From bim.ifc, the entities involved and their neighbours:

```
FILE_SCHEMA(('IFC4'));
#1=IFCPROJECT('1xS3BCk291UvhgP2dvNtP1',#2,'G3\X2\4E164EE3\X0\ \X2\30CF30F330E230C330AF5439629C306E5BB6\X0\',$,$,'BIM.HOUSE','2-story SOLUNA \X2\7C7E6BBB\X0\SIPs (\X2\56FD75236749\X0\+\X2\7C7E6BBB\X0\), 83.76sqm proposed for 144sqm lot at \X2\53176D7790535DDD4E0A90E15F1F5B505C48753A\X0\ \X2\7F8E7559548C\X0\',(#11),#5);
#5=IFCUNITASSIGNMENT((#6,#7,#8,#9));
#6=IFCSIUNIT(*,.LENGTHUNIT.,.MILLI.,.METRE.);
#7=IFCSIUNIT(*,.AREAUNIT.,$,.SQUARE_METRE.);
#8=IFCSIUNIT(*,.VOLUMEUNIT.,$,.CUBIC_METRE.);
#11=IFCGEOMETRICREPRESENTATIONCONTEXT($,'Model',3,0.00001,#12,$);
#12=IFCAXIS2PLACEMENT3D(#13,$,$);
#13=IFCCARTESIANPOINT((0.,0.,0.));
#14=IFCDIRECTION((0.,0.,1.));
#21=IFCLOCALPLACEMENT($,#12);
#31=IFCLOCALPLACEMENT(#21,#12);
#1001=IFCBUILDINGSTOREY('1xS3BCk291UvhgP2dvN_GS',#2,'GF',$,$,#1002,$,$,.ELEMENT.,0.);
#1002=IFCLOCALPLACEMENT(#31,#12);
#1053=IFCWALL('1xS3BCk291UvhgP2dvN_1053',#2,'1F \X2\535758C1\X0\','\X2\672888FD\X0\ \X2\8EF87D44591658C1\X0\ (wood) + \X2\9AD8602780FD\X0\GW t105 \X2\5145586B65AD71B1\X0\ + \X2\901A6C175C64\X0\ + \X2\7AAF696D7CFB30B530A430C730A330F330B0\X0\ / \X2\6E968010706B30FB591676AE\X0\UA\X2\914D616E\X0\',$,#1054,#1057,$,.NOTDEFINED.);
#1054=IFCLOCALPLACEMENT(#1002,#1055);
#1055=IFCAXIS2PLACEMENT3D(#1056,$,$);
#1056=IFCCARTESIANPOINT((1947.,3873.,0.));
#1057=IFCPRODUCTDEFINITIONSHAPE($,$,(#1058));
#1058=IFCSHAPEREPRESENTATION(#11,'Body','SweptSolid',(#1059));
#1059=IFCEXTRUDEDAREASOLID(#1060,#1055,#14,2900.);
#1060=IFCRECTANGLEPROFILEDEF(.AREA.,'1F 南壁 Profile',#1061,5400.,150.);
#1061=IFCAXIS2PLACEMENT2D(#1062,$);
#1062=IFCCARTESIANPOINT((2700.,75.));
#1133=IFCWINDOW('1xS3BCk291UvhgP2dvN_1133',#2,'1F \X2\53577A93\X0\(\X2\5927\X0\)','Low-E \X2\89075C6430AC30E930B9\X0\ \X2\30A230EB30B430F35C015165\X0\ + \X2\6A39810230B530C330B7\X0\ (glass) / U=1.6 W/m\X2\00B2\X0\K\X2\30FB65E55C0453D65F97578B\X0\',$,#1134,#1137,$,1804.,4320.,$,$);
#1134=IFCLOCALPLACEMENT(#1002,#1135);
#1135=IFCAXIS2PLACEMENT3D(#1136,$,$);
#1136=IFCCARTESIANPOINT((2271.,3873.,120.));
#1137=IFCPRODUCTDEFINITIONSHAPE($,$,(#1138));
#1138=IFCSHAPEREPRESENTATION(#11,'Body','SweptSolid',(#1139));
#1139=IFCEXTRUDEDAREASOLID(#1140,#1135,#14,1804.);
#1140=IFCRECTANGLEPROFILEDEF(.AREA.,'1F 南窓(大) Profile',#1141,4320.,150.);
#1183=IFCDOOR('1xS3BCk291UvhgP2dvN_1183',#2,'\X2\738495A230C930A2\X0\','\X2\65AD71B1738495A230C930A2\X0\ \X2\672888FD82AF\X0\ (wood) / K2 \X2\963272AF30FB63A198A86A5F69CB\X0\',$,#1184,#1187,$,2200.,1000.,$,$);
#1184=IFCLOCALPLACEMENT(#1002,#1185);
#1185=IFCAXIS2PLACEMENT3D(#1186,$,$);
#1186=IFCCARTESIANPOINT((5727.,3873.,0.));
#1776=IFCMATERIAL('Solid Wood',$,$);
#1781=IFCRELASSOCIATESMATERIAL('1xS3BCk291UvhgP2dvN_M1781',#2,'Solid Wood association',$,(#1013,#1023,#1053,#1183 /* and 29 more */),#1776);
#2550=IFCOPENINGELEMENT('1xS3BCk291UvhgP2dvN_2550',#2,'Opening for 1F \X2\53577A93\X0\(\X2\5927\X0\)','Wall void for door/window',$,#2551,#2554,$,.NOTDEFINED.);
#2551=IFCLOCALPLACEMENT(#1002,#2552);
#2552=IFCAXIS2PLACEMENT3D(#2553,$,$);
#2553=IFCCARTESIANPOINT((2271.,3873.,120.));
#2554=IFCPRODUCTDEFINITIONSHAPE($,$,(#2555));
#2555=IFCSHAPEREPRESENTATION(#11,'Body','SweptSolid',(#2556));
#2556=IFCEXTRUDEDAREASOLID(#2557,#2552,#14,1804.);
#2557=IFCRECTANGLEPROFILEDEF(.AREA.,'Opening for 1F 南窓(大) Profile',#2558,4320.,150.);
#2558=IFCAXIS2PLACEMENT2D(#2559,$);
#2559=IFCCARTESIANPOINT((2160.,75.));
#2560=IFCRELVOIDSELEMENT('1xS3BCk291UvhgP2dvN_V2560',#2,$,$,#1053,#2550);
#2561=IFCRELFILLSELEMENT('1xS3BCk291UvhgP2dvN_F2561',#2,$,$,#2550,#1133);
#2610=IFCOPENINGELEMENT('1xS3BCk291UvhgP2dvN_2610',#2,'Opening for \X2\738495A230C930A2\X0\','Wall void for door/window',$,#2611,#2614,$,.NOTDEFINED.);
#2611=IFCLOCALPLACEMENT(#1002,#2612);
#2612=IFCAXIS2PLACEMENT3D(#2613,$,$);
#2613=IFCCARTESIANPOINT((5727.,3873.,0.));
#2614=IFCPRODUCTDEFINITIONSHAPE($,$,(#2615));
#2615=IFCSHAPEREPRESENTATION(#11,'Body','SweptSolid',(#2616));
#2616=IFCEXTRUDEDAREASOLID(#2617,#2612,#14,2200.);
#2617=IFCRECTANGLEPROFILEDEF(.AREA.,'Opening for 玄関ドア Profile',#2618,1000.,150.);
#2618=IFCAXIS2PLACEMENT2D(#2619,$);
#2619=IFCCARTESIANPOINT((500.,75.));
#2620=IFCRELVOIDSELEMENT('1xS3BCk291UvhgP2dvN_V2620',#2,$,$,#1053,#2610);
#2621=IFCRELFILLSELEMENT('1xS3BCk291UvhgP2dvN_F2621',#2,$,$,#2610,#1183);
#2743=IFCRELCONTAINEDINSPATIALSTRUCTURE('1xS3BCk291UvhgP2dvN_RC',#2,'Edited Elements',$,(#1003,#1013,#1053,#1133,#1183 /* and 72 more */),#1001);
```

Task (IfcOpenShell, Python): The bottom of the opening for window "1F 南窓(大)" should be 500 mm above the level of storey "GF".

```python
import numpy as np
import ifcopenshell
import ifcopenshell.api.geometry
import ifcopenshell.geom
import ifcopenshell.util.element
import ifcopenshell.util.placement
import ifcopenshell.util.shape
import ifcopenshell.util.unit

model = ifcopenshell.open("bim.ifc")
unit_scale = ifcopenshell.util.unit.calculate_unit_scale(model)

window = model.by_guid("1xS3BCk291UvhgP2dvN_1133")
opening = window.FillsVoids[0].RelatingOpeningElement
storey = ifcopenshell.util.element.get_container(window, ifc_class="IfcBuildingStorey")
level = ifcopenshell.util.placement.get_local_placement(storey.ObjectPlacement)[2, 3]

# The opening's origin need not be at the sill, so measure its lowest point.
shape = ifcopenshell.geom.create_shape(ifcopenshell.geom.settings(), opening)
bottom = ifcopenshell.util.shape.get_shape_bottom_elevation(shape, shape.geometry) / unit_scale
dz = level + 0.5 / unit_scale - bottom

shift = np.array([0.0, 0.0, dz])
# The window is not placed relative to its opening, so move both.
for product in (opening, window):
    matrix = ifcopenshell.util.placement.get_local_placement(product.ObjectPlacement)
    matrix[:3, 3] += shift
    ifcopenshell.api.geometry.edit_object_placement(model, product=product, matrix=matrix, is_si=False)

print(f"moved by {dz * unit_scale:+.3f} m")

model.write("bim_v2.ifc")
```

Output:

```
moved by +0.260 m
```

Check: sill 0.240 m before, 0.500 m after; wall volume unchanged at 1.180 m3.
